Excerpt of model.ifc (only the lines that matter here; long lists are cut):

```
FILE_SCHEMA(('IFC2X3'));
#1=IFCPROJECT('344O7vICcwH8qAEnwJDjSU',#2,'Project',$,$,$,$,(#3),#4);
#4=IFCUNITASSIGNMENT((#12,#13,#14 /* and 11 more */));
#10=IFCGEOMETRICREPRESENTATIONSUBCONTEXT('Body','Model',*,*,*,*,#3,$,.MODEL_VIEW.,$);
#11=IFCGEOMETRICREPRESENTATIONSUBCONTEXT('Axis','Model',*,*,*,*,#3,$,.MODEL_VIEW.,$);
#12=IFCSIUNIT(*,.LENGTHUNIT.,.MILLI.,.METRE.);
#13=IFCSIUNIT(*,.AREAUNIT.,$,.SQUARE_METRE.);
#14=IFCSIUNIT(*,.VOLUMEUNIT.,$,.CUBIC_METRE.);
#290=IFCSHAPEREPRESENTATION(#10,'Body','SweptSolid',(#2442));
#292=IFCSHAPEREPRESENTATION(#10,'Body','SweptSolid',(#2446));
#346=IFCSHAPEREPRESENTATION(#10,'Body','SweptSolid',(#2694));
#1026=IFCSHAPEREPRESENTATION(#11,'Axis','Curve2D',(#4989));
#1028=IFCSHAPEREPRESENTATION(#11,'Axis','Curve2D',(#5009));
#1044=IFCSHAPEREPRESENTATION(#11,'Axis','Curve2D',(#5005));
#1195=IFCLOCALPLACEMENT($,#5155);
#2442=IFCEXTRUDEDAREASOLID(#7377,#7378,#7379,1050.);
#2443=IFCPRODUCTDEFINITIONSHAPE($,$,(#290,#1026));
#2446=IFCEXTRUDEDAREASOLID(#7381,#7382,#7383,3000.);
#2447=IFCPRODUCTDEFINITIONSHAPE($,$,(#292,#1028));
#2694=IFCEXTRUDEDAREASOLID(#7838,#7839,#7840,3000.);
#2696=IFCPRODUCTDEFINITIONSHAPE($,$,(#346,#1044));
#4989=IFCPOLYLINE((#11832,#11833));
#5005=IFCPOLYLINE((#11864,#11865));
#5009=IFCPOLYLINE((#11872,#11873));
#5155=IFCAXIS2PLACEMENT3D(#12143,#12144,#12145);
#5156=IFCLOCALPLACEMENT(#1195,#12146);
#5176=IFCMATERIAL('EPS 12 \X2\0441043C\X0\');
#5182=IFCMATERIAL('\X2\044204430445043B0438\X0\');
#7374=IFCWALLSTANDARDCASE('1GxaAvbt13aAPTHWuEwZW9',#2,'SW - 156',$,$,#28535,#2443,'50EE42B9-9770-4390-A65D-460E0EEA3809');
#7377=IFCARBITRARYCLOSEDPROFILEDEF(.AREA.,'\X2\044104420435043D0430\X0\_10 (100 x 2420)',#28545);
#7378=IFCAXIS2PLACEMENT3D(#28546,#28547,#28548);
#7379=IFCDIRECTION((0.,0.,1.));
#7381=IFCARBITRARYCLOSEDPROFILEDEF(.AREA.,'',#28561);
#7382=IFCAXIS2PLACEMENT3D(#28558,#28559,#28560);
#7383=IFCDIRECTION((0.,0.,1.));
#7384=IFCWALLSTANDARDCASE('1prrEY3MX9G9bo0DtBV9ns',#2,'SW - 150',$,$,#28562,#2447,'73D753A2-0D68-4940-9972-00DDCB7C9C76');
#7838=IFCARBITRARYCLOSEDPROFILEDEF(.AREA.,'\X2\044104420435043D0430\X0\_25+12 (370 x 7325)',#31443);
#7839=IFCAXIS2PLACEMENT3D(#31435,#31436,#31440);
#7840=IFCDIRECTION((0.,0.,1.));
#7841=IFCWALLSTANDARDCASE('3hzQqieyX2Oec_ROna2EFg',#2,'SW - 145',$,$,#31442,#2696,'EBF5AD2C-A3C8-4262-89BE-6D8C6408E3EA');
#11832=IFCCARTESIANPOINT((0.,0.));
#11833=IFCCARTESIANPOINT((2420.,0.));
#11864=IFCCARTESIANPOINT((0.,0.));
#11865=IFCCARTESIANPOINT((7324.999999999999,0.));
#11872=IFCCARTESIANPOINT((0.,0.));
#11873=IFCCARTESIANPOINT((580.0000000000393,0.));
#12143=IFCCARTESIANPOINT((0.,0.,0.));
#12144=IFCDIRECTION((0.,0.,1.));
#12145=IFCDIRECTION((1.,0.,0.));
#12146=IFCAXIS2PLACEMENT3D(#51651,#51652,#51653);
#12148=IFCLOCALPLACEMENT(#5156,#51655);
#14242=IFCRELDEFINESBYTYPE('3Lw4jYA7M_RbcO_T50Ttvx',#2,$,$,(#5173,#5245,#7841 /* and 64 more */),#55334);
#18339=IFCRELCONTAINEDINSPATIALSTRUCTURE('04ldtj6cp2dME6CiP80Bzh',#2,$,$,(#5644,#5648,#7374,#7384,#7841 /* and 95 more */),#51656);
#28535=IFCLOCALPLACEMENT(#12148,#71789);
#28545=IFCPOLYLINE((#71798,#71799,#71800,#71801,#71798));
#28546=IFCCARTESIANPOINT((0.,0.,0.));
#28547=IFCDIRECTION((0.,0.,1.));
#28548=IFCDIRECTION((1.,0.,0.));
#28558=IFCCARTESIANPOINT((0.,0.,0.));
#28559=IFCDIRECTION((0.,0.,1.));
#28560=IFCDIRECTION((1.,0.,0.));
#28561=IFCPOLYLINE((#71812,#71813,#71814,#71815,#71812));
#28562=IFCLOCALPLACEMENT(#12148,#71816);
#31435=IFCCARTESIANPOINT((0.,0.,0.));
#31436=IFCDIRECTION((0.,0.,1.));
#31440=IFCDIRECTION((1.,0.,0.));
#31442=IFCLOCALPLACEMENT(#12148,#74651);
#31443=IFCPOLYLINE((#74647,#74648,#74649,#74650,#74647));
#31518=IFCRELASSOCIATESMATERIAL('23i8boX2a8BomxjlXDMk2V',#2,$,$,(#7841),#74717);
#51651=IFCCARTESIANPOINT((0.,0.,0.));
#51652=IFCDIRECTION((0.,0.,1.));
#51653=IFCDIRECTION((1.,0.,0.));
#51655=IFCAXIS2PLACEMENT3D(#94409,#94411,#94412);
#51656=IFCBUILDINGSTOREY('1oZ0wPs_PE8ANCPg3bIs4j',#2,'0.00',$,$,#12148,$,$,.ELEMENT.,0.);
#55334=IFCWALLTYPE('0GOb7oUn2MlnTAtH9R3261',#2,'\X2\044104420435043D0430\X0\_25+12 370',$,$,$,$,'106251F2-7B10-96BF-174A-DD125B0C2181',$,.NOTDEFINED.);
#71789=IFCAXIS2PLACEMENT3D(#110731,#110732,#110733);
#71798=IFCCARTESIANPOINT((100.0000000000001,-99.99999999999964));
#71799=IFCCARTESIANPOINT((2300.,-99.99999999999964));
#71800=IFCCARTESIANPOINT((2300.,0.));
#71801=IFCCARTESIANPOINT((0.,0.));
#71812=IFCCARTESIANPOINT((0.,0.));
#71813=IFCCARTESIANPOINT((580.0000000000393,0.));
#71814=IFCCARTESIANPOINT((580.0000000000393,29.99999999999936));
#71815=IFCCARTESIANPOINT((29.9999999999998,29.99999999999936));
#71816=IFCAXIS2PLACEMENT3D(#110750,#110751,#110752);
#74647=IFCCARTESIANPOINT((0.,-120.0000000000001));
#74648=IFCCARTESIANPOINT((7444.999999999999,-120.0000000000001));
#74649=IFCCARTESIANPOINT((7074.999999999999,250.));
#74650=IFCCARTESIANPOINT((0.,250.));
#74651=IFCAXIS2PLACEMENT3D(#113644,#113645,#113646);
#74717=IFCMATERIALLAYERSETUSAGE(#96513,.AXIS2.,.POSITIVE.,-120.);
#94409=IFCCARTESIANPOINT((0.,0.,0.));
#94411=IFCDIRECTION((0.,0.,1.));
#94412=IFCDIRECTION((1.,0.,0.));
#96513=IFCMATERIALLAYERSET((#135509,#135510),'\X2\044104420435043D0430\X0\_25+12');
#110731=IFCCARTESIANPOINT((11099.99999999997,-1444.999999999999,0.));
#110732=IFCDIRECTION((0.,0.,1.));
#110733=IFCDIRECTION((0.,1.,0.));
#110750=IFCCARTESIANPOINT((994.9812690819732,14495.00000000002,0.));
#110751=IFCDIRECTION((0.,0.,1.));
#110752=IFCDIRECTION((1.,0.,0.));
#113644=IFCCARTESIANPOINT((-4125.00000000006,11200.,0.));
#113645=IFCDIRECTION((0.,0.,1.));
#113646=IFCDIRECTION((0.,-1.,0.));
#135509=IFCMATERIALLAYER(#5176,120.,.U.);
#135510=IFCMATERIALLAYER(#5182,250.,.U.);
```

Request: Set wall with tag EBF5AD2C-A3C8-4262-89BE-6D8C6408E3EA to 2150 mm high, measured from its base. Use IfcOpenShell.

```python
import ifcopenshell
import ifcopenshell.geom
import ifcopenshell.util.representation
import ifcopenshell.util.shape

model = ifcopenshell.open("model.ifc")
settings = ifcopenshell.geom.settings()


def volume(element):
    """Net volume in cubic metres, openings subtracted."""
    shape = ifcopenshell.geom.create_shape(settings, element)
    return ifcopenshell.util.shape.get_volume(shape.geometry)


wall = model.by_guid("3hzQqieyX2Oec_ROna2EFg")
before = volume(wall)

body = ifcopenshell.util.representation.get_representation(wall, "Model", "Body")
solid = body.Items[0]
old_height = solid.Depth
solid.Depth = 2150.0
after = volume(wall)

print(f"height {old_height:g} -> {solid.Depth:g}, volume {before:.3f} -> {after:.3f} m3")

model.write("model-out.ifc")
```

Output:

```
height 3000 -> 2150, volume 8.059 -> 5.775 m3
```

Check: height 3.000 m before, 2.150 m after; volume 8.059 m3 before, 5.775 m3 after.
